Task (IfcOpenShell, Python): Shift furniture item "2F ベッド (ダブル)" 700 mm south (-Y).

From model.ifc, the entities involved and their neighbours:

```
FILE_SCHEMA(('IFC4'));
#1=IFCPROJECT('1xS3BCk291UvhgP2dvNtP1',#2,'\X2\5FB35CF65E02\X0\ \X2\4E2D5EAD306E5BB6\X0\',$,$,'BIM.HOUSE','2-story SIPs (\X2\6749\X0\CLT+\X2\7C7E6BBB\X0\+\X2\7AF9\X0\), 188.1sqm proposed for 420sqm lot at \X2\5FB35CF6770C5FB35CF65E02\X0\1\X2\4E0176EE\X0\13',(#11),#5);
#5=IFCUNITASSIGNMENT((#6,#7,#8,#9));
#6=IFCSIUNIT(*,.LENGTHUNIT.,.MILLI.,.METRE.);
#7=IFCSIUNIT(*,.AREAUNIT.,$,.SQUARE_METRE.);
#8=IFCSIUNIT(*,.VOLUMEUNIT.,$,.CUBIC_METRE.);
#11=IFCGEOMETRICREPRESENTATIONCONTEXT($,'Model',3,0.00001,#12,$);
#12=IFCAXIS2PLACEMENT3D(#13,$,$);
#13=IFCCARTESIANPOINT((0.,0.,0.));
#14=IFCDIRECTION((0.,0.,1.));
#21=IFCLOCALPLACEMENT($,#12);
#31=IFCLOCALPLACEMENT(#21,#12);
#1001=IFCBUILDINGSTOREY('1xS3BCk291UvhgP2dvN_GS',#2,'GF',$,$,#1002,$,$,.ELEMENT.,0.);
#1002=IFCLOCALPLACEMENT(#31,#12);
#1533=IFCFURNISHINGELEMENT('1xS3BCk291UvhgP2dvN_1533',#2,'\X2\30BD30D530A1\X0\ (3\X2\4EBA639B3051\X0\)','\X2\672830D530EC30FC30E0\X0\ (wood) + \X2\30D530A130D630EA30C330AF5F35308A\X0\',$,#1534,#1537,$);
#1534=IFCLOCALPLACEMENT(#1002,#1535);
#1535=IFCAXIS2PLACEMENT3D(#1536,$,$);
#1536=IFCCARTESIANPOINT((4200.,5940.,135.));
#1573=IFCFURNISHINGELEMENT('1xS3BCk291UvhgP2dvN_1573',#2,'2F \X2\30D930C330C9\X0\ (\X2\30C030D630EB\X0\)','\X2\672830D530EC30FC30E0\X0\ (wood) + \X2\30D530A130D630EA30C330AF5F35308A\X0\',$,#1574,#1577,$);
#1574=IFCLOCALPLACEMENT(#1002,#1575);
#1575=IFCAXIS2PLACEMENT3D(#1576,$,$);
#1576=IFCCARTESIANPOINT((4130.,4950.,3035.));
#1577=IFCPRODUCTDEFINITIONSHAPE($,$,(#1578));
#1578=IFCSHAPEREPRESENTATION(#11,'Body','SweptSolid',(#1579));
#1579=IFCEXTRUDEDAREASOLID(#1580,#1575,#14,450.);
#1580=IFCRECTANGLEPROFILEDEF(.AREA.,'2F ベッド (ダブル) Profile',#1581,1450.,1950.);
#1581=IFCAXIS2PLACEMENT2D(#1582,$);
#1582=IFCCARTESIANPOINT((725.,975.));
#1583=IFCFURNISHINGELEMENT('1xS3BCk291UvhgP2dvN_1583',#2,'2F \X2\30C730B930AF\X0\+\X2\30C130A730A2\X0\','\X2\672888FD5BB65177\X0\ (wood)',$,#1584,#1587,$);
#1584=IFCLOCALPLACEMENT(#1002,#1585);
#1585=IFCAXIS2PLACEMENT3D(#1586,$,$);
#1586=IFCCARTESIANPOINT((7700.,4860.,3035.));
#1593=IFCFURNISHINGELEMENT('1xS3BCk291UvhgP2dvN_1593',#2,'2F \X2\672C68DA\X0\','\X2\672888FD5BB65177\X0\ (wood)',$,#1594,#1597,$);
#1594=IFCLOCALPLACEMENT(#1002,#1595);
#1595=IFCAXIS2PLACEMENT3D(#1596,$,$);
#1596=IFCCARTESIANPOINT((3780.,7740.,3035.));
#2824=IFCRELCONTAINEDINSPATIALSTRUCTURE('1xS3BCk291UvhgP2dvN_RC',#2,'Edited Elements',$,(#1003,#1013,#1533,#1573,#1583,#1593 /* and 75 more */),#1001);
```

```python
import ifcopenshell
import ifcopenshell.api.geometry
import ifcopenshell.util.placement
import ifcopenshell.util.unit

model = ifcopenshell.open("model.ifc")
unit_scale = ifcopenshell.util.unit.calculate_unit_scale(model)

item = model.by_guid("1xS3BCk291UvhgP2dvN_1573")
matrix = ifcopenshell.util.placement.get_local_placement(item.ObjectPlacement)
matrix[1, 3] -= 0.7 / unit_scale
ifcopenshell.api.geometry.edit_object_placement(model, product=item, matrix=matrix, is_si=False)

print(ifcopenshell.util.placement.get_local_placement(item.ObjectPlacement).round(3) + 0.0)

model.write("model_rev.ifc")
```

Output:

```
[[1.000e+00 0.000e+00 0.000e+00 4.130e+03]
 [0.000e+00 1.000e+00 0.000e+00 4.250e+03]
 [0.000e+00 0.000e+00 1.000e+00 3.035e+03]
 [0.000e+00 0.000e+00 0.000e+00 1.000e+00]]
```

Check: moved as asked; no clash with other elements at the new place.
